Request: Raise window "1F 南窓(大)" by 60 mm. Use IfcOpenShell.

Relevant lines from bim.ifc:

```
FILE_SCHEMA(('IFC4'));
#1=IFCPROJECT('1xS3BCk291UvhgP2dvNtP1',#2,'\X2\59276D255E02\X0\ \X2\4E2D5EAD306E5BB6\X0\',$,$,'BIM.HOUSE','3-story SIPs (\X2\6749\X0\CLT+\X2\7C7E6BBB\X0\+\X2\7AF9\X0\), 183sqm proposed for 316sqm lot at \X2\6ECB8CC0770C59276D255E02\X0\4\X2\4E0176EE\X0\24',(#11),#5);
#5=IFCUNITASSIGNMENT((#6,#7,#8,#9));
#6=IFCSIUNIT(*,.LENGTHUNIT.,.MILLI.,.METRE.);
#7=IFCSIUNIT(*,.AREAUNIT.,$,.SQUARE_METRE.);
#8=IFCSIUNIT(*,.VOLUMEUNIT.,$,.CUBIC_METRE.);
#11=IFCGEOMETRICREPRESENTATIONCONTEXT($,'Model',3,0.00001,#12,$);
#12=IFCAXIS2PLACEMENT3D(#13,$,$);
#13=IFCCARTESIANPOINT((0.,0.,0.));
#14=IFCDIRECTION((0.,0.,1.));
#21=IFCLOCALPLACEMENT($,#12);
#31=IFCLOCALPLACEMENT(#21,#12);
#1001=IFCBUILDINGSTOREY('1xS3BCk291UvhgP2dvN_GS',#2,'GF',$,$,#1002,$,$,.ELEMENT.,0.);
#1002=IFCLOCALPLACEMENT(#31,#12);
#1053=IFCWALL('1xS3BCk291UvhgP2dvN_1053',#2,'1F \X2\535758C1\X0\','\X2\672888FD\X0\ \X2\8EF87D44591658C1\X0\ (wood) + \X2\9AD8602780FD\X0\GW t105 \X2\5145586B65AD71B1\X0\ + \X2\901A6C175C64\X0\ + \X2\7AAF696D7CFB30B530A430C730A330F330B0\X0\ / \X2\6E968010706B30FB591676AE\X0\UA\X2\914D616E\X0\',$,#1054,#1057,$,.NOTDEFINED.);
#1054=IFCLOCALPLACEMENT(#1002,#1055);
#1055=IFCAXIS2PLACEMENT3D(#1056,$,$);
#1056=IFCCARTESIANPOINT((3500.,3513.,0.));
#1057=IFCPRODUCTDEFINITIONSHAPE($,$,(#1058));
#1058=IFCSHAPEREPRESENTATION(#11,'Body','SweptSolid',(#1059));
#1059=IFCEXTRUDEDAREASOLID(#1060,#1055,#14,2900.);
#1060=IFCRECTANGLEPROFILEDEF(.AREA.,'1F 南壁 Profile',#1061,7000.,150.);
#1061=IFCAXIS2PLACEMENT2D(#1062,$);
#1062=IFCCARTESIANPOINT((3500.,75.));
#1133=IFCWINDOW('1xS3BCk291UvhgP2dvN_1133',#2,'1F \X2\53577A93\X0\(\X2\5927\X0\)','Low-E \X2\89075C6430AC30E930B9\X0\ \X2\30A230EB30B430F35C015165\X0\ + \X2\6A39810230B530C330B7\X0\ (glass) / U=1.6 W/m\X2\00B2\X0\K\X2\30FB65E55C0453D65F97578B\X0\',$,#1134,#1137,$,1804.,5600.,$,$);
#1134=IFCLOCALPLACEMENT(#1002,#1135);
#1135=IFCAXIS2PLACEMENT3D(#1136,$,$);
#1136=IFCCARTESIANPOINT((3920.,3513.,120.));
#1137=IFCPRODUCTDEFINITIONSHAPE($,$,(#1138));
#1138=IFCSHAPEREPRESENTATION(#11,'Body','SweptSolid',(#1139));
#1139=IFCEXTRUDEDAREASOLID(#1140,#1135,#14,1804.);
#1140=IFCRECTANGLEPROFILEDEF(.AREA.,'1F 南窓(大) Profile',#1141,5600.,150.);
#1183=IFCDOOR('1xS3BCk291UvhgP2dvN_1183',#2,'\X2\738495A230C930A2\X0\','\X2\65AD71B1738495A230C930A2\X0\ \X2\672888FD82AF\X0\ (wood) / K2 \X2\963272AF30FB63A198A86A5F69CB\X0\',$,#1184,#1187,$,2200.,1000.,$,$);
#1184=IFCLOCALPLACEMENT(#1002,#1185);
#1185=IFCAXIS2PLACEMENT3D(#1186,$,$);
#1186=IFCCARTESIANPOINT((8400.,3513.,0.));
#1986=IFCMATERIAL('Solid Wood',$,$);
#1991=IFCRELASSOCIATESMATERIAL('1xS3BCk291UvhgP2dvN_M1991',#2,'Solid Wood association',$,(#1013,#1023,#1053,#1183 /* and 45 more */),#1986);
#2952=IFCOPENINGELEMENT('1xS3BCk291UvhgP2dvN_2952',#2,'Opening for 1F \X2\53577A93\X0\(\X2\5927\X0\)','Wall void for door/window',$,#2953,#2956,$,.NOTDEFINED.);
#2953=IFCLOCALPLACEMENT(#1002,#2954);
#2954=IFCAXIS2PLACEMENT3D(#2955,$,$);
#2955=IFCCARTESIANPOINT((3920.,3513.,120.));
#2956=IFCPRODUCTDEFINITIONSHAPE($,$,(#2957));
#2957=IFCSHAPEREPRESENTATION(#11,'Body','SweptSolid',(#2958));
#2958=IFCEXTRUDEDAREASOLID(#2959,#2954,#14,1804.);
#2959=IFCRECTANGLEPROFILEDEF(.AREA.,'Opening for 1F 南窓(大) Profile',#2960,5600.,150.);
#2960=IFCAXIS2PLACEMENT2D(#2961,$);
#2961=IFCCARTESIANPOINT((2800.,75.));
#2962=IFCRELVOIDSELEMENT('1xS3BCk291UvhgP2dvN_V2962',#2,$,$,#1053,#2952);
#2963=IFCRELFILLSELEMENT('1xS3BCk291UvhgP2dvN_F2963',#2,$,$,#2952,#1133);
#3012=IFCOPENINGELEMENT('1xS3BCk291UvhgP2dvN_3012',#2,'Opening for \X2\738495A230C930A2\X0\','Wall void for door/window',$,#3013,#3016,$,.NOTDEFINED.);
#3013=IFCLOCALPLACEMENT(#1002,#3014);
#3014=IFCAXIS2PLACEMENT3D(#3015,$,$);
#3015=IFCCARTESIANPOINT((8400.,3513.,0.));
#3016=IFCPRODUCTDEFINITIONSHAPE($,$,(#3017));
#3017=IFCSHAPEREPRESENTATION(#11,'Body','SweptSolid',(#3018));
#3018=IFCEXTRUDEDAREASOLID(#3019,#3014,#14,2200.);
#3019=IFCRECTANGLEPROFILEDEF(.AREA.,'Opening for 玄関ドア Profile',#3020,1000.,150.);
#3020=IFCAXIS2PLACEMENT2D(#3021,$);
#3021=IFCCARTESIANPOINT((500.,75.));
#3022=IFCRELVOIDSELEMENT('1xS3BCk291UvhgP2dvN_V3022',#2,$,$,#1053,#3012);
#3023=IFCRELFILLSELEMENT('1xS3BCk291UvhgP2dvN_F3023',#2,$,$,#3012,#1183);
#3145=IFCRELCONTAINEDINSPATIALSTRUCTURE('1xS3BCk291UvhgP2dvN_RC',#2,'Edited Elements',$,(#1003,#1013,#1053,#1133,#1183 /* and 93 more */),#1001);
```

```python
import numpy as np
import ifcopenshell
import ifcopenshell.api.geometry
import ifcopenshell.util.placement
import ifcopenshell.util.unit

model = ifcopenshell.open("bim.ifc")
unit_scale = ifcopenshell.util.unit.calculate_unit_scale(model)

window = model.by_guid("1xS3BCk291UvhgP2dvN_1133")
opening = window.FillsVoids[0].RelatingOpeningElement
dz = 0.06 / unit_scale

shift = np.array([0.0, 0.0, dz])
# The window is not placed relative to its opening, so move both.
for product in (opening, window):
    matrix = ifcopenshell.util.placement.get_local_placement(product.ObjectPlacement)
    matrix[:3, 3] += shift
    ifcopenshell.api.geometry.edit_object_placement(model, product=product, matrix=matrix, is_si=False)

print(f"moved by {dz * unit_scale:+.3f} m")

model.write("bim_updated.ifc")
```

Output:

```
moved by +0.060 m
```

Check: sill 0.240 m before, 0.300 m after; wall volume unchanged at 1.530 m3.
